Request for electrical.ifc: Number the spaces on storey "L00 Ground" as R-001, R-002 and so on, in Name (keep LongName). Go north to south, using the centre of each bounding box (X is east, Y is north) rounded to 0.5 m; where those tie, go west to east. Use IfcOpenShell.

First a look at what the model holds.

```python
import ifcopenshell
import ifcopenshell.util.element
import ifcopenshell.util.placement

model = ifcopenshell.open("electrical.ifc")
print(model.schema)
storey = next(s for s in model.by_type("IfcBuildingStorey") if s.Name == "L00 Ground")
spaces = [e for e in ifcopenshell.util.element.get_decomposition(storey) if e.is_a("IfcSpace")]
for e in sorted(spaces, key=lambda e: e.id()):
    origin = ifcopenshell.util.placement.get_local_placement(e.ObjectPlacement)[:3, 3]
    print(e.id(), e.Name, e.LongName, origin.round(2) + 0.0, sep=" | ")
```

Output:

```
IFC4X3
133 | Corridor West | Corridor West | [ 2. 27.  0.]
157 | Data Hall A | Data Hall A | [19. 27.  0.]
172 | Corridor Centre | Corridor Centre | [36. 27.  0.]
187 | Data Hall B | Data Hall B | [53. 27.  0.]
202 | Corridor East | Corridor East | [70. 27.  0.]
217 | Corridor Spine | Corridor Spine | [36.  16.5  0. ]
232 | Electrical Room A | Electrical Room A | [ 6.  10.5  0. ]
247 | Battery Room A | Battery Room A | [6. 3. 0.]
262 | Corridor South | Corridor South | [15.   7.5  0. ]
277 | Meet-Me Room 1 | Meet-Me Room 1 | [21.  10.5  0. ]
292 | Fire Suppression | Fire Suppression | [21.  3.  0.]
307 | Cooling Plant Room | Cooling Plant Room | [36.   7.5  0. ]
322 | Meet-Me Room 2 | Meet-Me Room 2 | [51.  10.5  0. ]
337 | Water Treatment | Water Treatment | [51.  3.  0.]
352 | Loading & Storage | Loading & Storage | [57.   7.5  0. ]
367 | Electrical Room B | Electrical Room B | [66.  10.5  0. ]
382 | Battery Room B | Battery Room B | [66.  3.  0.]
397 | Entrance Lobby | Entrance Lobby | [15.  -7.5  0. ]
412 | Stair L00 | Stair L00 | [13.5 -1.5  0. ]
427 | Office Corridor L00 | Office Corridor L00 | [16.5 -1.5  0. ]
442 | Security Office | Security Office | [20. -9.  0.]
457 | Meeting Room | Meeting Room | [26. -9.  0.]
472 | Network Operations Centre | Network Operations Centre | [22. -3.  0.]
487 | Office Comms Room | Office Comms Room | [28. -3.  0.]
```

```python
import ifcopenshell
import ifcopenshell.geom
import ifcopenshell.util.element
import ifcopenshell.util.shape

model = ifcopenshell.open("electrical.ifc")
settings = ifcopenshell.geom.settings()
settings.set("use-world-coords", True)


def centre(element):
    shape = ifcopenshell.geom.create_shape(settings, element)
    return ifcopenshell.util.shape.get_bbox_centroid(shape.geometry)


storey = next(s for s in model.by_type("IfcBuildingStorey") if s.Name == "L00 Ground")
spaces = [e for e in ifcopenshell.util.element.get_decomposition(storey) if e.is_a("IfcSpace")]

# Insertion points can sit at a corner or the storey origin, so sort by the geometry (in metres).
centres = {e: centre(e) for e in spaces}
spaces.sort(key=lambda e: (-round(centres[e][1] / 0.5), centres[e][0]))

for i, e in enumerate(spaces, start=1):
    number = f"R-0{i:02d}"
    e.Name = number
    print(e.id(), number)

model.write("electrical-out.ifc")
```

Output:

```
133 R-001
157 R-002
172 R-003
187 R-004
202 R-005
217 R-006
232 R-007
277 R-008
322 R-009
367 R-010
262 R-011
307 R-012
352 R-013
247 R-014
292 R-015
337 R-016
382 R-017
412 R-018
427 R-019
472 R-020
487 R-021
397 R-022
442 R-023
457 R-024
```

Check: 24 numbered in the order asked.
